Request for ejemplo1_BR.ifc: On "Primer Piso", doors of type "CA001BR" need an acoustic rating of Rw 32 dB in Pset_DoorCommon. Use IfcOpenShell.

First a look at what the model holds.

```python
import ifcopenshell
import ifcopenshell.util.element

model = ifcopenshell.open("ejemplo1_BR.ifc")
print(model.schema)
storey = next(s for s in model.by_type("IfcBuildingStorey") if s.Name == "Primer Piso")
doors = [e for e in ifcopenshell.util.element.get_decomposition(storey) if e.is_a("IfcDoor")]
seen = {}
for e in doors:
    element_type = ifcopenshell.util.element.get_type(e)
    key = (element_type.Name if element_type != e and element_type else None, ifcopenshell.util.element.get_pset(e, "Pset_DoorCommon", "AcousticRating"))
    seen[key] = seen.get(key, 0) + 1
for (name, value), count in sorted(seen.items(), key=str):
    print(count, "x", name, "|", value)
```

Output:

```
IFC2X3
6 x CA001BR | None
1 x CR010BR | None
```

```python
import ifcopenshell
import ifcopenshell.api.pset
import ifcopenshell.util.element

model = ifcopenshell.open("ejemplo1_BR.ifc")

storey = next(s for s in model.by_type("IfcBuildingStorey") if s.Name == "Primer Piso")
doors = [e for e in ifcopenshell.util.element.get_decomposition(storey) if e.is_a("IfcDoor")]

count = 0
for e in doors:
    element_type = ifcopenshell.util.element.get_type(e)
    if element_type in (None, e) or element_type.Name != "CA001BR":
        continue
    # add_pset returns the element's existing set when there is one.
    pset = ifcopenshell.api.pset.add_pset(model, product=e, name="Pset_DoorCommon")
    ifcopenshell.api.pset.edit_pset(model, pset=pset, properties={"AcousticRating": "Rw 32 dB"})
    count += 1

print(count, "doors updated")

model.write("ejemplo1_BR_v2.ifc")
```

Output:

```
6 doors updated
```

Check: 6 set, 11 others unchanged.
